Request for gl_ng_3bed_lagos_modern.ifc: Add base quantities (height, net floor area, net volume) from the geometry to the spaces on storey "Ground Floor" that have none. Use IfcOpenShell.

First a look at what the model holds.

```python
import ifcopenshell
import ifcopenshell.util.element
import ifcopenshell.util.unit

model = ifcopenshell.open("gl_ng_3bed_lagos_modern.ifc")
print(model.schema)
for unit_type in ("LENGTHUNIT", "AREAUNIT", "VOLUMEUNIT"):
    print(unit_type, ifcopenshell.util.unit.calculate_unit_scale(model, unit_type))
storey = next(s for s in model.by_type("IfcBuildingStorey") if s.Name == "Ground Floor")
spaces = [e for e in ifcopenshell.util.element.get_decomposition(storey) if e.is_a("IfcSpace")]
for e in sorted(spaces, key=lambda e: e.id()):
    print(e.id(), e.is_a(), e.Name, list(ifcopenshell.util.element.get_psets(e, qtos_only=True)), sep=" | ")
```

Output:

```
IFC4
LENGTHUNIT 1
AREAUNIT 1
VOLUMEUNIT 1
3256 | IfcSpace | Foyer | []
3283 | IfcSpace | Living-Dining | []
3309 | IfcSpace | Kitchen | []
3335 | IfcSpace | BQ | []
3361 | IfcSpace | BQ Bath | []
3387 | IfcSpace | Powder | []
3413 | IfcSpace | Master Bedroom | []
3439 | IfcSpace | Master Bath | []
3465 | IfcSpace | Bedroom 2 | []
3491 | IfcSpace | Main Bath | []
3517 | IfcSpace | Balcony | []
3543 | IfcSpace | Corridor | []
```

```python
import ifcopenshell
import ifcopenshell.api.pset
import ifcopenshell.geom
import ifcopenshell.util.element
import ifcopenshell.util.shape
import ifcopenshell.util.unit

model = ifcopenshell.open("gl_ng_3bed_lagos_modern.ifc")
unit_scale = ifcopenshell.util.unit.calculate_unit_scale(model)
area_scale = ifcopenshell.util.unit.calculate_unit_scale(model, "AREAUNIT")
volume_scale = ifcopenshell.util.unit.calculate_unit_scale(model, "VOLUMEUNIT")
settings = ifcopenshell.geom.settings()

storey = next(s for s in model.by_type("IfcBuildingStorey") if s.Name == "Ground Floor")
spaces = [e for e in ifcopenshell.util.element.get_decomposition(storey) if e.is_a("IfcSpace")]

for e in sorted(spaces, key=lambda e: e.id()):
    if ifcopenshell.util.element.get_psets(e, qtos_only=True, should_inherit=False):
        continue
    # Geometry comes back in metres, in the element's own axes.
    shape = ifcopenshell.geom.create_shape(settings, e)
    values = {
        "Height": ifcopenshell.util.shape.get_z(shape.geometry) / unit_scale,
        "NetFloorArea": ifcopenshell.util.shape.get_footprint_area(shape.geometry) / area_scale,
        "NetVolume": ifcopenshell.util.shape.get_volume(shape.geometry) / volume_scale,
    }
    qto = ifcopenshell.api.pset.add_qto(model, product=e, name="Qto_SpaceBaseQuantities")
    ifcopenshell.api.pset.edit_qto(model, qto=qto, properties=values)
    print(e.id(), {k: round(v, 3) for k, v in values.items()})

model.write("gl_ng_3bed_lagos_modern_updated.ifc")
```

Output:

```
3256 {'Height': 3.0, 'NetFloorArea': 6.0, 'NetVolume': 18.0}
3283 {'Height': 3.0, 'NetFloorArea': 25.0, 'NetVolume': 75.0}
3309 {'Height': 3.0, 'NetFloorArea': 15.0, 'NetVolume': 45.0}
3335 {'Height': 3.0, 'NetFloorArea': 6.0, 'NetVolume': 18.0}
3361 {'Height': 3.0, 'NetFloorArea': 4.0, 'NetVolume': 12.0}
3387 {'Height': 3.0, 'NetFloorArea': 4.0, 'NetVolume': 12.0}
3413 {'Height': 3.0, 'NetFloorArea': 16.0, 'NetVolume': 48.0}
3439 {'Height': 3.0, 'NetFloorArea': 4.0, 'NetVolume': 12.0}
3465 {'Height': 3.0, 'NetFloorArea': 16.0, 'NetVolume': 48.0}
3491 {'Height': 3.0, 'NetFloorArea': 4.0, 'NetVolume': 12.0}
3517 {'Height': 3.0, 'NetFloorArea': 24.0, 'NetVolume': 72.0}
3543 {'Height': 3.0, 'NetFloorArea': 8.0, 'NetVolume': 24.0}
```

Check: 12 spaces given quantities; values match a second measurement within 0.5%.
